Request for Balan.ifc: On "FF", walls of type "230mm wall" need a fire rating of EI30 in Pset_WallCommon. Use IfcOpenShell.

First a look at what the model holds.

```python
import ifcopenshell
import ifcopenshell.util.element

model = ifcopenshell.open("Balan.ifc")
print(model.schema)
storey = next(s for s in model.by_type("IfcBuildingStorey") if s.Name == "FF")
walls = [e for e in ifcopenshell.util.element.get_decomposition(storey) if e.is_a("IfcWall")]
seen = {}
for e in walls:
    element_type = ifcopenshell.util.element.get_type(e)
    key = (element_type.Name if element_type != e and element_type else None, ifcopenshell.util.element.get_pset(e, "Pset_WallCommon", "FireRating"))
    seen[key] = seen.get(key, 0) + 1
for (name, value), count in sorted(seen.items(), key=str):
    print(count, "x", name, "|", value)
```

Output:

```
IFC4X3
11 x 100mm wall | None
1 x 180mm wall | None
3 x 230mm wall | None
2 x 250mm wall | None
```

```python
import ifcopenshell
import ifcopenshell.api.pset
import ifcopenshell.util.element

model = ifcopenshell.open("Balan.ifc")

storey = next(s for s in model.by_type("IfcBuildingStorey") if s.Name == "FF")
walls = [e for e in ifcopenshell.util.element.get_decomposition(storey) if e.is_a("IfcWall")]

count = 0
for e in walls:
    element_type = ifcopenshell.util.element.get_type(e)
    if element_type in (None, e) or element_type.Name != "230mm wall":
        continue
    # add_pset returns the element's existing set when there is one.
    pset = ifcopenshell.api.pset.add_pset(model, product=e, name="Pset_WallCommon")
    ifcopenshell.api.pset.edit_pset(model, pset=pset, properties={"FireRating": "EI30"})
    count += 1

print(count, "walls updated")

model.write("Balan_updated.ifc")
```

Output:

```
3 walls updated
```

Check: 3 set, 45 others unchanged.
